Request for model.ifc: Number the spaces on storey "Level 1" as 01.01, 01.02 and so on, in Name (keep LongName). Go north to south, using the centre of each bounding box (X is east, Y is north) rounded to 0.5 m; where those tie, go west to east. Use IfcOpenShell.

First a look at what the model holds.

```python
import ifcopenshell
import ifcopenshell.util.element
import ifcopenshell.util.placement

model = ifcopenshell.open("model.ifc")
print(model.schema)
storey = next(s for s in model.by_type("IfcBuildingStorey") if s.Name == "Level 1")
spaces = [e for e in ifcopenshell.util.element.get_decomposition(storey) if e.is_a("IfcSpace")]
for e in sorted(spaces, key=lambda e: e.id()):
    origin = ifcopenshell.util.placement.get_local_placement(e.ObjectPlacement)[:3, 3]
    print(e.id(), e.Name, e.LongName, origin.round(2) + 0.0, sep=" | ")
```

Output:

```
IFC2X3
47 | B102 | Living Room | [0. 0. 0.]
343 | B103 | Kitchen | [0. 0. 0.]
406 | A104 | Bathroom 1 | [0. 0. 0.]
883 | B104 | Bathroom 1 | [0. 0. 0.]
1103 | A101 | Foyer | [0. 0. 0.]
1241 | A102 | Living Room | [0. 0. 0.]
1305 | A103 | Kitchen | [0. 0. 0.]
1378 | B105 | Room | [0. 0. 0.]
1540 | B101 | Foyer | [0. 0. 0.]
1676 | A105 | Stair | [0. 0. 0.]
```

```python
import ifcopenshell
import ifcopenshell.geom
import ifcopenshell.util.element
import ifcopenshell.util.shape

model = ifcopenshell.open("model.ifc")
settings = ifcopenshell.geom.settings()
settings.set("use-world-coords", True)


def centre(element):
    shape = ifcopenshell.geom.create_shape(settings, element)
    return ifcopenshell.util.shape.get_bbox_centroid(shape.geometry)


storey = next(s for s in model.by_type("IfcBuildingStorey") if s.Name == "Level 1")
spaces = [e for e in ifcopenshell.util.element.get_decomposition(storey) if e.is_a("IfcSpace")]

# Insertion points can sit at a corner or the storey origin, so sort by the geometry (in metres).
centres = {e: centre(e) for e in spaces}
spaces.sort(key=lambda e: (-round(centres[e][1] / 0.5), centres[e][0]))

for i, e in enumerate(spaces, start=1):
    number = f"01.{i:02d}"
    e.Name = number
    print(e.id(), number)

model.write("model_updated.ifc")
```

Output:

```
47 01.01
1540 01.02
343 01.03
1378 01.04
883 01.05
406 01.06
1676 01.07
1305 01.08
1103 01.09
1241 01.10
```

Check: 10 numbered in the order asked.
